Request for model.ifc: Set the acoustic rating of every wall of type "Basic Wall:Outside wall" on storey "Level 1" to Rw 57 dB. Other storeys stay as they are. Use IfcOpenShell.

First a look at what the model holds.

```python
import ifcopenshell
import ifcopenshell.util.element

model = ifcopenshell.open("model.ifc")
print(model.schema)
storey = next(s for s in model.by_type("IfcBuildingStorey") if s.Name == "Level 1")
walls = [e for e in ifcopenshell.util.element.get_decomposition(storey) if e.is_a("IfcWall")]
seen = {}
for e in walls:
    element_type = ifcopenshell.util.element.get_type(e)
    key = (element_type.Name if element_type != e and element_type else None, ifcopenshell.util.element.get_pset(e, "Pset_WallCommon", "AcousticRating"))
    seen[key] = seen.get(key, 0) + 1
for (name, value), count in sorted(seen.items(), key=str):
    print(count, "x", name, "|", value)
```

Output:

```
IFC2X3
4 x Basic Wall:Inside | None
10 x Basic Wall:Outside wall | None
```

```python
import ifcopenshell
import ifcopenshell.api.pset
import ifcopenshell.util.element

model = ifcopenshell.open("model.ifc")

storey = next(s for s in model.by_type("IfcBuildingStorey") if s.Name == "Level 1")
walls = [e for e in ifcopenshell.util.element.get_decomposition(storey) if e.is_a("IfcWall")]

count = 0
for e in walls:
    element_type = ifcopenshell.util.element.get_type(e)
    if element_type in (None, e) or element_type.Name != "Basic Wall:Outside wall":
        continue
    # add_pset returns the element's existing set when there is one.
    pset = ifcopenshell.api.pset.add_pset(model, product=e, name="Pset_WallCommon")
    ifcopenshell.api.pset.edit_pset(model, pset=pset, properties={"AcousticRating": "Rw 57 dB"})
    count += 1

print(count, "walls updated")

model.write("model_updated.ifc")
```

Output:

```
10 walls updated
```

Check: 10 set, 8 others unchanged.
